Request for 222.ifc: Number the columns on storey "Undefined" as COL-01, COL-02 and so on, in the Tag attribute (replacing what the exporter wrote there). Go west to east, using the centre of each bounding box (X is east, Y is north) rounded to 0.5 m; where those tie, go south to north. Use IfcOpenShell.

First a look at what the model holds.

```python
import ifcopenshell
import ifcopenshell.util.element
import ifcopenshell.util.placement

model = ifcopenshell.open("222.ifc")
print(model.schema)
storey = next(s for s in model.by_type("IfcBuildingStorey") if s.Name == "Undefined")
columns = [e for e in ifcopenshell.util.element.get_decomposition(storey) if e.is_a("IfcColumn")]
for e in sorted(columns, key=lambda e: e.id()):
    origin = ifcopenshell.util.placement.get_local_placement(e.ObjectPlacement)[:3, 3]
    print(e.id(), e.Tag, e.Name, origin.round(2) + 0.0, sep=" | ")
```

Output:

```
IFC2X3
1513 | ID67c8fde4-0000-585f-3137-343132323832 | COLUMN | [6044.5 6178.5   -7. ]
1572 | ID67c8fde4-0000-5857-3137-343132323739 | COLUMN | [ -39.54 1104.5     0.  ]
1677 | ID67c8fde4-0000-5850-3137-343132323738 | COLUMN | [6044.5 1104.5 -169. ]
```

```python
import ifcopenshell
import ifcopenshell.geom
import ifcopenshell.util.element
import ifcopenshell.util.shape

model = ifcopenshell.open("222.ifc")
settings = ifcopenshell.geom.settings()
settings.set("use-world-coords", True)


def centre(element):
    shape = ifcopenshell.geom.create_shape(settings, element)
    return ifcopenshell.util.shape.get_bbox_centroid(shape.geometry)


storey = next(s for s in model.by_type("IfcBuildingStorey") if s.Name == "Undefined")
columns = [e for e in ifcopenshell.util.element.get_decomposition(storey) if e.is_a("IfcColumn")]

# Insertion points can sit at a corner or the storey origin, so sort by the geometry (in metres).
centres = {e: centre(e) for e in columns}
columns.sort(key=lambda e: (round(centres[e][0] / 0.5), centres[e][1]))

for i, e in enumerate(columns, start=1):
    number = f"COL-{i:02d}"
    e.Tag = number
    print(e.id(), number)

model.write("222_updated.ifc")
```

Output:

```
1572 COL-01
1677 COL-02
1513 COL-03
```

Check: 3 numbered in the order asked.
